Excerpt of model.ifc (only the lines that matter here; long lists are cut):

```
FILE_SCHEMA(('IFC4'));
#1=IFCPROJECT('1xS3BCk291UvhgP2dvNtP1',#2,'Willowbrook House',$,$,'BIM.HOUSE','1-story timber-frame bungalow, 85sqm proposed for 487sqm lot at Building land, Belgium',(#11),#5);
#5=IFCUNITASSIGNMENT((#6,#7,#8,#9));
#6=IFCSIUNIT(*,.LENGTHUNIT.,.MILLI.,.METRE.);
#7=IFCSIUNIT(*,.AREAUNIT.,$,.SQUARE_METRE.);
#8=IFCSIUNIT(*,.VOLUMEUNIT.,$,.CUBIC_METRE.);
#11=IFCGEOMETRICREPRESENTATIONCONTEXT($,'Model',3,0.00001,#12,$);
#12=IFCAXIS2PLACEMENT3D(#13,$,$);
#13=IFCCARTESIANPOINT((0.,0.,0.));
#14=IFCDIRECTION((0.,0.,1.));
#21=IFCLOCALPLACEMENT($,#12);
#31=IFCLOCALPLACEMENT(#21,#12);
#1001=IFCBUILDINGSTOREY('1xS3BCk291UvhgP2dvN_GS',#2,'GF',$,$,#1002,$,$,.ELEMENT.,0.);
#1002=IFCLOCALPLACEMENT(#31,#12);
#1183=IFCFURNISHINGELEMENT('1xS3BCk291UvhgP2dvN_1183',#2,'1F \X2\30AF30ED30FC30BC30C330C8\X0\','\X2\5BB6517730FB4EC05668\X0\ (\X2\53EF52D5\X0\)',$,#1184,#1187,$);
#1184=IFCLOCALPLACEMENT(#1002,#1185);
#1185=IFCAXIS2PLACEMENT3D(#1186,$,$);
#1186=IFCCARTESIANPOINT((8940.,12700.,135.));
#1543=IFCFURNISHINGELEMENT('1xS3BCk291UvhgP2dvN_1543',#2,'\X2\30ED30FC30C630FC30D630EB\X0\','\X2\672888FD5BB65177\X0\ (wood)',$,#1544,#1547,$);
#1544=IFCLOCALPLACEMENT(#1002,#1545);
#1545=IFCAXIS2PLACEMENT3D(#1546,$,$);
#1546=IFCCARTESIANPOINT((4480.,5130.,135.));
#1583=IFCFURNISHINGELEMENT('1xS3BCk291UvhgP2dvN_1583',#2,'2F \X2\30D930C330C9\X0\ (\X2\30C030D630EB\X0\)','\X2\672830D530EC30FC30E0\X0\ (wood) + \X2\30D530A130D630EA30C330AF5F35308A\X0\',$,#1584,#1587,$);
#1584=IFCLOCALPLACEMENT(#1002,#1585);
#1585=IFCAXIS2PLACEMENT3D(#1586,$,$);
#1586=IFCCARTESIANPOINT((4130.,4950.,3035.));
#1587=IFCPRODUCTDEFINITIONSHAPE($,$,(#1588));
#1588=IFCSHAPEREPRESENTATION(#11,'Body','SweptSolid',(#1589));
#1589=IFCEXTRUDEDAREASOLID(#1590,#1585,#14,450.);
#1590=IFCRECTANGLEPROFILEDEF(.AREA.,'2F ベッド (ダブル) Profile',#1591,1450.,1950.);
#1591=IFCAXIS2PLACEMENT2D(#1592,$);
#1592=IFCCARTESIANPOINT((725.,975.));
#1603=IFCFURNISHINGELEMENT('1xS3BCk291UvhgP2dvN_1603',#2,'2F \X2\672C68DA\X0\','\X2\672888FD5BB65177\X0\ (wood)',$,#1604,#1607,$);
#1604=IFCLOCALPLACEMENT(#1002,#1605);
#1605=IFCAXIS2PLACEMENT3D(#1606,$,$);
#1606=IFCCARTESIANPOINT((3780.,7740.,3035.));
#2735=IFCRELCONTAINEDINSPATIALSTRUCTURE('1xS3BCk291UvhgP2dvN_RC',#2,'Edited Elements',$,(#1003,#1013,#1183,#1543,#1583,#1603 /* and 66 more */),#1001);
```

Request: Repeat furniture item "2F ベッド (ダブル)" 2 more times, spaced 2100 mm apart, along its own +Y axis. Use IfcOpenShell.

```python
import ifcopenshell
import ifcopenshell.api.geometry
import ifcopenshell.api.root
import ifcopenshell.util.element
import ifcopenshell.util.placement

model = ifcopenshell.open("model.ifc")


def reuse_history(source, copy):
    """copy_class also copies each property set's owner history, people and application; keep the originals."""
    for rel in copy.IsDefinedBy:
        if rel.is_a("IfcRelDefinesByProperties") and (history := rel.RelatingPropertyDefinition.OwnerHistory):
            rel.RelatingPropertyDefinition.OwnerHistory = source.OwnerHistory
            ifcopenshell.util.element.remove_deep2(model, history)


source = model.by_id(1583)
base = ifcopenshell.util.placement.get_local_placement(source.ObjectPlacement)
step = base[:3, 1] * 2100.0

for i in range(1, 3):
    copy = ifcopenshell.api.root.copy_class(model, product=source)
    copy.Representation = ifcopenshell.util.element.copy_deep(
        model, source.Representation, exclude=["IfcGeometricRepresentationContext", "IfcRepresentationMap"]
    )
    reuse_history(source, copy)
    matrix = base.copy()
    matrix[:3, 3] += i * step
    print("added at", matrix[:3, 3].round(3) + 0.0)
    ifcopenshell.api.geometry.edit_object_placement(model, product=copy, matrix=matrix, is_si=False)

model.write("model_updated.ifc")
```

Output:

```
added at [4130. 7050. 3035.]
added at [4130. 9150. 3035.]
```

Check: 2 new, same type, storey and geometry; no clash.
